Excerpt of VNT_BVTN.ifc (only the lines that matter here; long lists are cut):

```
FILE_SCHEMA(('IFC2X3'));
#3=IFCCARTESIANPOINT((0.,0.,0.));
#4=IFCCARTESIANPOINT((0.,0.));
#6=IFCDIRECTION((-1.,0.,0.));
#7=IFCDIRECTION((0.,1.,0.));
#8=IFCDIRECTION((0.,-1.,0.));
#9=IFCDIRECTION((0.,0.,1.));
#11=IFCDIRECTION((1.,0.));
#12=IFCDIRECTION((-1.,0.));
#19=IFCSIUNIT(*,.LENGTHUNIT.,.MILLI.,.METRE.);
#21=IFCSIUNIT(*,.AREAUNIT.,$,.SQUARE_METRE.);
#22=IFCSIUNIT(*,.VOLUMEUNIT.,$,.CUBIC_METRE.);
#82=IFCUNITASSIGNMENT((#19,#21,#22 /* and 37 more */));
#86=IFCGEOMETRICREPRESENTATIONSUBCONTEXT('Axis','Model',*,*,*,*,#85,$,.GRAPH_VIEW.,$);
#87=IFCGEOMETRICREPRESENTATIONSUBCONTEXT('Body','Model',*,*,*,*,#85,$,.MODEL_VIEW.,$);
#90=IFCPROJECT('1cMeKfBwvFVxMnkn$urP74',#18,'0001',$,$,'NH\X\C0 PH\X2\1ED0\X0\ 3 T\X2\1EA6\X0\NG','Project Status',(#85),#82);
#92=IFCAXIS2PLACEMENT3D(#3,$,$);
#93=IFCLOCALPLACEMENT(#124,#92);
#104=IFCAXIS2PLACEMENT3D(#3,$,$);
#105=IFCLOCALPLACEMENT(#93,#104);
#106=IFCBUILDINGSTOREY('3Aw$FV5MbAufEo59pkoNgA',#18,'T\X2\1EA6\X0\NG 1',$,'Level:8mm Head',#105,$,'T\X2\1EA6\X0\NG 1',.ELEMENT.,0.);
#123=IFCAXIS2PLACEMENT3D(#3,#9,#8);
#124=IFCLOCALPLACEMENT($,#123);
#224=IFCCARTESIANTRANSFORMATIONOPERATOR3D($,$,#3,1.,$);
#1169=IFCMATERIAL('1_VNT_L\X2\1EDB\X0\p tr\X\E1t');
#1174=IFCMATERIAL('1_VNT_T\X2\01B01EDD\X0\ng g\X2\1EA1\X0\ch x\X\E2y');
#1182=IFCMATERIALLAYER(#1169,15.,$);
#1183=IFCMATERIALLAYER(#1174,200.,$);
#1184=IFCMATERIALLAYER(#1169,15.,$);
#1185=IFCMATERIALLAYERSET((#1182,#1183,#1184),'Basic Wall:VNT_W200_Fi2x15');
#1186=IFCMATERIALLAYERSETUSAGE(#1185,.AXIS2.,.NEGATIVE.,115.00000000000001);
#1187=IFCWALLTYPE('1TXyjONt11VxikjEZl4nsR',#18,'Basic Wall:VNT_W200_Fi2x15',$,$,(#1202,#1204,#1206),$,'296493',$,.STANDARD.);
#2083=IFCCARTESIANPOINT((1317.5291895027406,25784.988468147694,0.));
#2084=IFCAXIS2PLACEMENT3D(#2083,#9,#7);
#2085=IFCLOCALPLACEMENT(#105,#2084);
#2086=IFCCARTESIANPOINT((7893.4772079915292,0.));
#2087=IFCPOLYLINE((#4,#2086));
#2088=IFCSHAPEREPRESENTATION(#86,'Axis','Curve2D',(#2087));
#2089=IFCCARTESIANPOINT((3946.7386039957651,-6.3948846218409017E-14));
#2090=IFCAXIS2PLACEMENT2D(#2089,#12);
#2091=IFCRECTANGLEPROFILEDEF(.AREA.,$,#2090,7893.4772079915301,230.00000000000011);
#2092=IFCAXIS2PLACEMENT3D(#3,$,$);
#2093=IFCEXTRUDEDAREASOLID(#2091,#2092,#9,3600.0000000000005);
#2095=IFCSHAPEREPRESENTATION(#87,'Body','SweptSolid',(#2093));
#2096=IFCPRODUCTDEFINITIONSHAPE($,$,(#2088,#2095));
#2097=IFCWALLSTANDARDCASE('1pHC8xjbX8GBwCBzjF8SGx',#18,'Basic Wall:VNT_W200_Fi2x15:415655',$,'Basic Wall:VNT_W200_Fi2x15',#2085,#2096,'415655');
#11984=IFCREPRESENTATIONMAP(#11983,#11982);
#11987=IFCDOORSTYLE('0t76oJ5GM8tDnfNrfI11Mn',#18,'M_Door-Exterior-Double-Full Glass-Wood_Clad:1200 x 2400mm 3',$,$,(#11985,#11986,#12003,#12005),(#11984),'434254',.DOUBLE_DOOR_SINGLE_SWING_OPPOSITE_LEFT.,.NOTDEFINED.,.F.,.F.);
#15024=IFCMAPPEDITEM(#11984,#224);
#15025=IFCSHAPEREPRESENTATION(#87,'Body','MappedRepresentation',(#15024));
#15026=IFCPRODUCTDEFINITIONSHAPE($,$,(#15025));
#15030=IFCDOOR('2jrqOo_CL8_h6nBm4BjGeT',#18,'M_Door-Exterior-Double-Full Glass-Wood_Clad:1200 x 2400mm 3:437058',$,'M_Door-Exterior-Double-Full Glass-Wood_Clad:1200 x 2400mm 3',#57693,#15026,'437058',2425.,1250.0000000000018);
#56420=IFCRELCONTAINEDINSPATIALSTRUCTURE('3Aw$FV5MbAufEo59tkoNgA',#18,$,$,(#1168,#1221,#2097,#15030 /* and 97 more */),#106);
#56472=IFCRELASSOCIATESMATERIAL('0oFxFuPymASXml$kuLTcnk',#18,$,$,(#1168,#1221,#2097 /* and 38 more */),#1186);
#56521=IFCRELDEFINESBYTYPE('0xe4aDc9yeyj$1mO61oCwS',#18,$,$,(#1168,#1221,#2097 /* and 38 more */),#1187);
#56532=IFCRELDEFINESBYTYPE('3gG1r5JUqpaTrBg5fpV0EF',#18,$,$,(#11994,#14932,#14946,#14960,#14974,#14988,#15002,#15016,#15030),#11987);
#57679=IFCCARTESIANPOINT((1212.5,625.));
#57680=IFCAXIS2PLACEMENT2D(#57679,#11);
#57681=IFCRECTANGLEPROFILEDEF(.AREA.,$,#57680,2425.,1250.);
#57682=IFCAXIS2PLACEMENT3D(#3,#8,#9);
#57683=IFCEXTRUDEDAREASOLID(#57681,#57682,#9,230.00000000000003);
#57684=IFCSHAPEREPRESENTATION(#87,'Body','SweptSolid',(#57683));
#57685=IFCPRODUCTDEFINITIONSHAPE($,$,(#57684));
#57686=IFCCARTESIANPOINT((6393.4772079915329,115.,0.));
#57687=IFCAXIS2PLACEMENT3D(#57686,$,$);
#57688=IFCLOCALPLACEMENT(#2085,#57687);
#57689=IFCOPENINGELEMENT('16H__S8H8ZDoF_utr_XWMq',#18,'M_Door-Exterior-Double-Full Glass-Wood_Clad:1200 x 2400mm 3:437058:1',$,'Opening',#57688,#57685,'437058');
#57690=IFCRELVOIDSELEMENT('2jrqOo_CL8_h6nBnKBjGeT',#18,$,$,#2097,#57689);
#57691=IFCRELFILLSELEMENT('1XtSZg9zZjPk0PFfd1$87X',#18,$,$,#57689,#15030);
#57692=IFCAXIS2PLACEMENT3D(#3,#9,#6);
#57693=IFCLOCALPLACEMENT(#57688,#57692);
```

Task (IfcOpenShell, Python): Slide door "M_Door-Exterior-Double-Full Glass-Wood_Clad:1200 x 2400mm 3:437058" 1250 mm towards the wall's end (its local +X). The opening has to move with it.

```python
import ifcopenshell
import ifcopenshell.api.geometry
import ifcopenshell.util.placement
import ifcopenshell.util.unit

model = ifcopenshell.open("VNT_BVTN.ifc")
unit_scale = ifcopenshell.util.unit.calculate_unit_scale(model)

door = model.by_guid("2jrqOo_CL8_h6nBm4BjGeT")
opening = door.FillsVoids[0].RelatingOpeningElement
wall = opening.VoidsElements[0].RelatingBuildingElement

wall_matrix = ifcopenshell.util.placement.get_local_placement(wall.ObjectPlacement)
shift = wall_matrix[:3, 0] * 1.25 / unit_scale
before = ifcopenshell.util.placement.get_local_placement(door.ObjectPlacement)[:3, 3].copy()

# The door is placed relative to its opening, so it follows when the opening moves.
matrix = ifcopenshell.util.placement.get_local_placement(opening.ObjectPlacement)
matrix[:3, 3] += shift
ifcopenshell.api.geometry.edit_object_placement(
    model, product=opening, matrix=matrix, is_si=False, should_transform_children=True
)

after = ifcopenshell.util.placement.get_local_placement(door.ObjectPlacement)[:3, 3]
print("door moved by", (after - before).round(3) + 0.0)

model.write("VNT_BVTN_v2.ifc")
```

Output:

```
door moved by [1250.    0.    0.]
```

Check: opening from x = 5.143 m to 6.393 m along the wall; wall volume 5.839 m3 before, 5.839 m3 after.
